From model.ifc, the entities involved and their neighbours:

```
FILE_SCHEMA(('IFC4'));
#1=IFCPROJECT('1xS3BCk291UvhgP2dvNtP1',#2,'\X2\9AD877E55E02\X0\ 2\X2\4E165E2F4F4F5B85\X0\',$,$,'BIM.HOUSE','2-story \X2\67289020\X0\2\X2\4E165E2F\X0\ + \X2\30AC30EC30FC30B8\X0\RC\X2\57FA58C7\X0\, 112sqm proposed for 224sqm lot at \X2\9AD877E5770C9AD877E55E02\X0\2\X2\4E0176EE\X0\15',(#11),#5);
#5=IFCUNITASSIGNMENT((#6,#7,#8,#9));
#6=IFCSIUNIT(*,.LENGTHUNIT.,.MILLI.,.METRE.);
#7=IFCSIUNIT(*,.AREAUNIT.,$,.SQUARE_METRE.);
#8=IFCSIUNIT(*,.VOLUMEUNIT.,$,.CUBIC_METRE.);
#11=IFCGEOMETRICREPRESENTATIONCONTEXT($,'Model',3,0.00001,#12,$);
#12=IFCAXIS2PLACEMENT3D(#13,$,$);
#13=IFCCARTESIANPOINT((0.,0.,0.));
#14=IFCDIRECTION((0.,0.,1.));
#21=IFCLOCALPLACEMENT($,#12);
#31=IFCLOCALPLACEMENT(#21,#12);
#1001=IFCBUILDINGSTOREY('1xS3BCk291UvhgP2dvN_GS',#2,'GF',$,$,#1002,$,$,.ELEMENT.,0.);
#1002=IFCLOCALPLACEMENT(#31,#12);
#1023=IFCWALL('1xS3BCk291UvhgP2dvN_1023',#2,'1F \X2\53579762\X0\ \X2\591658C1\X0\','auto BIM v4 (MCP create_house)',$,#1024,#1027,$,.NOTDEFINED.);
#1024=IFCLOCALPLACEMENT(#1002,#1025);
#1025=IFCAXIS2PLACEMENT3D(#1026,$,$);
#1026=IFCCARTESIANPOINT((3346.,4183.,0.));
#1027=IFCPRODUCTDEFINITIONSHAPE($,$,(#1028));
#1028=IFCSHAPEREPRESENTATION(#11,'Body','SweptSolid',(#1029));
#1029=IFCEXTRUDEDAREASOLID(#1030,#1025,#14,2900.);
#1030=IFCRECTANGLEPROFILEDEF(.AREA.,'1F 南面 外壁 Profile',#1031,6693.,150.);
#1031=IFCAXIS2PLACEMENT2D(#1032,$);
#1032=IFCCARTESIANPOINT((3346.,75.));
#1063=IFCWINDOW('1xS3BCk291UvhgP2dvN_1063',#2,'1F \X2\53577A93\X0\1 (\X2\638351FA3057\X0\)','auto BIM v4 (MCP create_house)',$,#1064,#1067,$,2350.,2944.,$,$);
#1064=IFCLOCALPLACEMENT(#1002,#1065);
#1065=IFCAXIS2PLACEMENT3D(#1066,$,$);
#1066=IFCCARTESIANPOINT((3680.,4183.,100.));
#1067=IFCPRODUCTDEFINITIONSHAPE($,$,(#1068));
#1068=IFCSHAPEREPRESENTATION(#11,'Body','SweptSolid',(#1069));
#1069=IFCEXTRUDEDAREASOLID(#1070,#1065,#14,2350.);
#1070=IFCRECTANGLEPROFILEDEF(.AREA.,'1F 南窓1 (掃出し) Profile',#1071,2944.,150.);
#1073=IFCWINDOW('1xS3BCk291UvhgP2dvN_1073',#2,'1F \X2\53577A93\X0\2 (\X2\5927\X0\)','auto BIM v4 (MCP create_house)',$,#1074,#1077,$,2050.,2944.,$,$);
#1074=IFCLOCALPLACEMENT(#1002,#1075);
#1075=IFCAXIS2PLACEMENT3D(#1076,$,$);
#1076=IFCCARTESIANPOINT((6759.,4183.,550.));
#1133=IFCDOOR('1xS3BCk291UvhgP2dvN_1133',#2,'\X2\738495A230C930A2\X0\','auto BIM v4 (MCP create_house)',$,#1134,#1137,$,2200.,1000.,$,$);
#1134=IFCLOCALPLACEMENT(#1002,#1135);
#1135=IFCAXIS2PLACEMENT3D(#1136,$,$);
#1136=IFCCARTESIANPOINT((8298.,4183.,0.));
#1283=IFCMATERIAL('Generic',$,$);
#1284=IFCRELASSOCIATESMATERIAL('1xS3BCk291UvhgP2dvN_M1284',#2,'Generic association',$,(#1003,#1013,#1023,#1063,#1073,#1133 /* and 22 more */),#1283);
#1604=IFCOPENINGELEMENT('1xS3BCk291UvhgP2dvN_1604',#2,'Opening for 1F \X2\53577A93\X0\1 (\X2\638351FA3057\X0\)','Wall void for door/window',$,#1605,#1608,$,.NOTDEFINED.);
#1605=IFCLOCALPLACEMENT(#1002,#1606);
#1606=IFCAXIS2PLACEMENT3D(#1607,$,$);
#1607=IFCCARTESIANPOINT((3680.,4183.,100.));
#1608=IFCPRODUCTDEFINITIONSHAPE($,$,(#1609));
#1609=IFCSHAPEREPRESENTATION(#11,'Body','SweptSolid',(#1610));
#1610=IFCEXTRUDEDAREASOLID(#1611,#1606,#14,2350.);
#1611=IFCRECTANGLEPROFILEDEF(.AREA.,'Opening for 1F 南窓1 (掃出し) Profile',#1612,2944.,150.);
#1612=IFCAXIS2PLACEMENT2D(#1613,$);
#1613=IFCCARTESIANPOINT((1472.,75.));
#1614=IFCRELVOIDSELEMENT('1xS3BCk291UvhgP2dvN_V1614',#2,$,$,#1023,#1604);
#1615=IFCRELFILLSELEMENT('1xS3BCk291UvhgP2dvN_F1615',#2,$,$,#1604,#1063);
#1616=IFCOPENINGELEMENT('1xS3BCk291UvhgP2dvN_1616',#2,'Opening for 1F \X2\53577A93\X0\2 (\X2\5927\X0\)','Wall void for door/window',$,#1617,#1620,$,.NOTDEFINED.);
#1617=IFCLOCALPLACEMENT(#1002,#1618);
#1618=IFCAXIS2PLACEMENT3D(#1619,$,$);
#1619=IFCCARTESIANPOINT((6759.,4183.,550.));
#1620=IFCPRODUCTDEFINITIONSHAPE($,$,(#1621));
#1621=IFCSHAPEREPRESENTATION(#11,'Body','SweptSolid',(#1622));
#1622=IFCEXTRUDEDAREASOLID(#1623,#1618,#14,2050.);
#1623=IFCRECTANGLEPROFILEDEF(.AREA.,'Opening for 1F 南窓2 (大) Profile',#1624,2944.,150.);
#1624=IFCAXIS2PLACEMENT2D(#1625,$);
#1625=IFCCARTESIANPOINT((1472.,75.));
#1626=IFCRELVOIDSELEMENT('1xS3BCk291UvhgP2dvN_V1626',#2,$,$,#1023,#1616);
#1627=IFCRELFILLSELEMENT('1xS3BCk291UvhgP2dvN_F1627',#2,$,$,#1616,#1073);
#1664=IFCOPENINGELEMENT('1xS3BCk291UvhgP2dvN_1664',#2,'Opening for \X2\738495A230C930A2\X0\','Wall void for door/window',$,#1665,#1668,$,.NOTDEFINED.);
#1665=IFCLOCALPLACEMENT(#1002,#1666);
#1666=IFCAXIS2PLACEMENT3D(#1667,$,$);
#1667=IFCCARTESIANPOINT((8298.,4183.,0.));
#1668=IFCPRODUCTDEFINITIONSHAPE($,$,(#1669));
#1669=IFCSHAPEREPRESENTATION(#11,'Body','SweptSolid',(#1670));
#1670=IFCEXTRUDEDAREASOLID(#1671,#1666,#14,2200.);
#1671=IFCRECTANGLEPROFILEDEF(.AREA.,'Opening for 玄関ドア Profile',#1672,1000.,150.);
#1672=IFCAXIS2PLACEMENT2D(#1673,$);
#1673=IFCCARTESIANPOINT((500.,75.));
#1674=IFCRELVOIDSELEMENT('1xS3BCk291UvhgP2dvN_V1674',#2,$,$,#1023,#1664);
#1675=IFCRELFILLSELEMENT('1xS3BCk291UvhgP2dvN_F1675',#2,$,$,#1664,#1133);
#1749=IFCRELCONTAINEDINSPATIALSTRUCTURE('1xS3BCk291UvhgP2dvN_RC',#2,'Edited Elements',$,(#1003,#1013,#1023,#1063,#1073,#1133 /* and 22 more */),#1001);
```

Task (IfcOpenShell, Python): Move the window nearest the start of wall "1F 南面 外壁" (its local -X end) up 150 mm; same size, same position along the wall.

```python
import numpy as np
import ifcopenshell
import ifcopenshell.api.geometry
import ifcopenshell.util.placement
import ifcopenshell.util.unit

model = ifcopenshell.open("model.ifc")
unit_scale = ifcopenshell.util.unit.calculate_unit_scale(model)

window = model.by_guid("1xS3BCk291UvhgP2dvN_1063")
opening = window.FillsVoids[0].RelatingOpeningElement
dz = 0.15 / unit_scale

shift = np.array([0.0, 0.0, dz])
# The window is not placed relative to its opening, so move both.
for product in (opening, window):
    matrix = ifcopenshell.util.placement.get_local_placement(product.ObjectPlacement)
    matrix[:3, 3] += shift
    ifcopenshell.api.geometry.edit_object_placement(model, product=product, matrix=matrix, is_si=False)

print(f"moved by {dz * unit_scale:+.3f} m")

model.write("model_edited.ifc")
```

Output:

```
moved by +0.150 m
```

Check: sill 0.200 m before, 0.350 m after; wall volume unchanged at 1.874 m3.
